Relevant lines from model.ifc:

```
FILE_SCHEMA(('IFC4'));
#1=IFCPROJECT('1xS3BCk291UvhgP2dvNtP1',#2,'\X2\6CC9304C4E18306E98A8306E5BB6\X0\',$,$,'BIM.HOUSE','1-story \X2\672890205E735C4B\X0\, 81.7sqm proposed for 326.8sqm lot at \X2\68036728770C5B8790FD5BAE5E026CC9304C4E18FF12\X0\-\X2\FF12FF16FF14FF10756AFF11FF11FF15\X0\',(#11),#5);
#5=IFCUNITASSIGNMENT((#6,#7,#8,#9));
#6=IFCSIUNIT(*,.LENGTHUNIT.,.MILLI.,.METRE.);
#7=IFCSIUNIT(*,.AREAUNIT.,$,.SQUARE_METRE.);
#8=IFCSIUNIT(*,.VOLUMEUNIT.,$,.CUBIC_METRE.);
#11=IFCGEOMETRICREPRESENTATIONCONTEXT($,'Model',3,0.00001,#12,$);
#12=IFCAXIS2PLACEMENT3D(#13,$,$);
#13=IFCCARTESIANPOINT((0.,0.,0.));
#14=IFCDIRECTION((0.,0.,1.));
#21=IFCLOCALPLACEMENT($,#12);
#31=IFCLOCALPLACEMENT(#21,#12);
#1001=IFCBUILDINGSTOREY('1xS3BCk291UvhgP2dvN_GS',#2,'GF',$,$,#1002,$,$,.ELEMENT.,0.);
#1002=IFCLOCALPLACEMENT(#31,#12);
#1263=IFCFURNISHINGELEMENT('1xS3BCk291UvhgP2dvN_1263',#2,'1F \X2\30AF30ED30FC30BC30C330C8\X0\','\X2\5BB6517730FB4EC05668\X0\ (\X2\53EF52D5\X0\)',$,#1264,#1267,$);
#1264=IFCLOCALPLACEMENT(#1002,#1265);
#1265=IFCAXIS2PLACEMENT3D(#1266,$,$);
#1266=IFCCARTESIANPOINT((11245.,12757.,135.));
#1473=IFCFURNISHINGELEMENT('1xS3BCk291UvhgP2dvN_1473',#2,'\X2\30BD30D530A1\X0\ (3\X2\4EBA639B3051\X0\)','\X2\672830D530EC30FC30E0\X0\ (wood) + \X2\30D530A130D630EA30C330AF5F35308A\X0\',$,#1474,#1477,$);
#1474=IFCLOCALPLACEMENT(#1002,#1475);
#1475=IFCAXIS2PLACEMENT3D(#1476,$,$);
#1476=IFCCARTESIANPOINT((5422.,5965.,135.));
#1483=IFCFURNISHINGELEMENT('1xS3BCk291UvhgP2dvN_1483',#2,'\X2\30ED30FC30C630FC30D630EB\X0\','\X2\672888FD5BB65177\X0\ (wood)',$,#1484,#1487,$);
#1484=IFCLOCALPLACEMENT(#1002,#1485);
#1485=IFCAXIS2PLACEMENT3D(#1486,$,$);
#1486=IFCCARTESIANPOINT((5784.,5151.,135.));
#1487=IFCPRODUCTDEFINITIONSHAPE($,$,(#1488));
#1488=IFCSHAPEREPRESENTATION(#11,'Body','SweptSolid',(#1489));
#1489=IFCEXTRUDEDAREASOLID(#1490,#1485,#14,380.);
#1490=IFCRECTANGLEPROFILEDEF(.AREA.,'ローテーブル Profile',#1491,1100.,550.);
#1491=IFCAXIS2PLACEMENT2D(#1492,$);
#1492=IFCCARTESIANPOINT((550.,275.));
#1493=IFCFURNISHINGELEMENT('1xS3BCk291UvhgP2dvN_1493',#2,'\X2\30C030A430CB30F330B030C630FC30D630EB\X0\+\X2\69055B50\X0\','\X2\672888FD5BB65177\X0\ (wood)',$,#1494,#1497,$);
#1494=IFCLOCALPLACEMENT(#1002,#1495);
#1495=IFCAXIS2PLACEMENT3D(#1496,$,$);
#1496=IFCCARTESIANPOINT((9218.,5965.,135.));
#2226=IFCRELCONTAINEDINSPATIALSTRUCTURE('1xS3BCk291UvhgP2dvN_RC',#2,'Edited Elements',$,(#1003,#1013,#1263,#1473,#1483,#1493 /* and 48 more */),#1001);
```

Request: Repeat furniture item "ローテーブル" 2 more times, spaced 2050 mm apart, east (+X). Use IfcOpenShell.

```python
import numpy as np
import ifcopenshell
import ifcopenshell.api.geometry
import ifcopenshell.api.root
import ifcopenshell.util.element
import ifcopenshell.util.placement

model = ifcopenshell.open("model.ifc")


def reuse_history(source, copy):
    """copy_class also copies each property set's owner history, people and application; keep the originals."""
    for rel in copy.IsDefinedBy:
        if rel.is_a("IfcRelDefinesByProperties") and (history := rel.RelatingPropertyDefinition.OwnerHistory):
            rel.RelatingPropertyDefinition.OwnerHistory = source.OwnerHistory
            ifcopenshell.util.element.remove_deep2(model, history)


source = model.by_guid("1xS3BCk291UvhgP2dvN_1483")
base = ifcopenshell.util.placement.get_local_placement(source.ObjectPlacement)
step = np.array([1.0, 0.0, 0.0]) * 2050.0

for i in range(1, 3):
    copy = ifcopenshell.api.root.copy_class(model, product=source)
    copy.Representation = ifcopenshell.util.element.copy_deep(
        model, source.Representation, exclude=["IfcGeometricRepresentationContext", "IfcRepresentationMap"]
    )
    reuse_history(source, copy)
    matrix = base.copy()
    matrix[:3, 3] += i * step
    print("added at", matrix[:3, 3].round(3) + 0.0)
    ifcopenshell.api.geometry.edit_object_placement(model, product=copy, matrix=matrix, is_si=False)

model.write("model_updated.ifc")
```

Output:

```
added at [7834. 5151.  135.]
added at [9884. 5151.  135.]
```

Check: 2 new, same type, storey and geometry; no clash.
